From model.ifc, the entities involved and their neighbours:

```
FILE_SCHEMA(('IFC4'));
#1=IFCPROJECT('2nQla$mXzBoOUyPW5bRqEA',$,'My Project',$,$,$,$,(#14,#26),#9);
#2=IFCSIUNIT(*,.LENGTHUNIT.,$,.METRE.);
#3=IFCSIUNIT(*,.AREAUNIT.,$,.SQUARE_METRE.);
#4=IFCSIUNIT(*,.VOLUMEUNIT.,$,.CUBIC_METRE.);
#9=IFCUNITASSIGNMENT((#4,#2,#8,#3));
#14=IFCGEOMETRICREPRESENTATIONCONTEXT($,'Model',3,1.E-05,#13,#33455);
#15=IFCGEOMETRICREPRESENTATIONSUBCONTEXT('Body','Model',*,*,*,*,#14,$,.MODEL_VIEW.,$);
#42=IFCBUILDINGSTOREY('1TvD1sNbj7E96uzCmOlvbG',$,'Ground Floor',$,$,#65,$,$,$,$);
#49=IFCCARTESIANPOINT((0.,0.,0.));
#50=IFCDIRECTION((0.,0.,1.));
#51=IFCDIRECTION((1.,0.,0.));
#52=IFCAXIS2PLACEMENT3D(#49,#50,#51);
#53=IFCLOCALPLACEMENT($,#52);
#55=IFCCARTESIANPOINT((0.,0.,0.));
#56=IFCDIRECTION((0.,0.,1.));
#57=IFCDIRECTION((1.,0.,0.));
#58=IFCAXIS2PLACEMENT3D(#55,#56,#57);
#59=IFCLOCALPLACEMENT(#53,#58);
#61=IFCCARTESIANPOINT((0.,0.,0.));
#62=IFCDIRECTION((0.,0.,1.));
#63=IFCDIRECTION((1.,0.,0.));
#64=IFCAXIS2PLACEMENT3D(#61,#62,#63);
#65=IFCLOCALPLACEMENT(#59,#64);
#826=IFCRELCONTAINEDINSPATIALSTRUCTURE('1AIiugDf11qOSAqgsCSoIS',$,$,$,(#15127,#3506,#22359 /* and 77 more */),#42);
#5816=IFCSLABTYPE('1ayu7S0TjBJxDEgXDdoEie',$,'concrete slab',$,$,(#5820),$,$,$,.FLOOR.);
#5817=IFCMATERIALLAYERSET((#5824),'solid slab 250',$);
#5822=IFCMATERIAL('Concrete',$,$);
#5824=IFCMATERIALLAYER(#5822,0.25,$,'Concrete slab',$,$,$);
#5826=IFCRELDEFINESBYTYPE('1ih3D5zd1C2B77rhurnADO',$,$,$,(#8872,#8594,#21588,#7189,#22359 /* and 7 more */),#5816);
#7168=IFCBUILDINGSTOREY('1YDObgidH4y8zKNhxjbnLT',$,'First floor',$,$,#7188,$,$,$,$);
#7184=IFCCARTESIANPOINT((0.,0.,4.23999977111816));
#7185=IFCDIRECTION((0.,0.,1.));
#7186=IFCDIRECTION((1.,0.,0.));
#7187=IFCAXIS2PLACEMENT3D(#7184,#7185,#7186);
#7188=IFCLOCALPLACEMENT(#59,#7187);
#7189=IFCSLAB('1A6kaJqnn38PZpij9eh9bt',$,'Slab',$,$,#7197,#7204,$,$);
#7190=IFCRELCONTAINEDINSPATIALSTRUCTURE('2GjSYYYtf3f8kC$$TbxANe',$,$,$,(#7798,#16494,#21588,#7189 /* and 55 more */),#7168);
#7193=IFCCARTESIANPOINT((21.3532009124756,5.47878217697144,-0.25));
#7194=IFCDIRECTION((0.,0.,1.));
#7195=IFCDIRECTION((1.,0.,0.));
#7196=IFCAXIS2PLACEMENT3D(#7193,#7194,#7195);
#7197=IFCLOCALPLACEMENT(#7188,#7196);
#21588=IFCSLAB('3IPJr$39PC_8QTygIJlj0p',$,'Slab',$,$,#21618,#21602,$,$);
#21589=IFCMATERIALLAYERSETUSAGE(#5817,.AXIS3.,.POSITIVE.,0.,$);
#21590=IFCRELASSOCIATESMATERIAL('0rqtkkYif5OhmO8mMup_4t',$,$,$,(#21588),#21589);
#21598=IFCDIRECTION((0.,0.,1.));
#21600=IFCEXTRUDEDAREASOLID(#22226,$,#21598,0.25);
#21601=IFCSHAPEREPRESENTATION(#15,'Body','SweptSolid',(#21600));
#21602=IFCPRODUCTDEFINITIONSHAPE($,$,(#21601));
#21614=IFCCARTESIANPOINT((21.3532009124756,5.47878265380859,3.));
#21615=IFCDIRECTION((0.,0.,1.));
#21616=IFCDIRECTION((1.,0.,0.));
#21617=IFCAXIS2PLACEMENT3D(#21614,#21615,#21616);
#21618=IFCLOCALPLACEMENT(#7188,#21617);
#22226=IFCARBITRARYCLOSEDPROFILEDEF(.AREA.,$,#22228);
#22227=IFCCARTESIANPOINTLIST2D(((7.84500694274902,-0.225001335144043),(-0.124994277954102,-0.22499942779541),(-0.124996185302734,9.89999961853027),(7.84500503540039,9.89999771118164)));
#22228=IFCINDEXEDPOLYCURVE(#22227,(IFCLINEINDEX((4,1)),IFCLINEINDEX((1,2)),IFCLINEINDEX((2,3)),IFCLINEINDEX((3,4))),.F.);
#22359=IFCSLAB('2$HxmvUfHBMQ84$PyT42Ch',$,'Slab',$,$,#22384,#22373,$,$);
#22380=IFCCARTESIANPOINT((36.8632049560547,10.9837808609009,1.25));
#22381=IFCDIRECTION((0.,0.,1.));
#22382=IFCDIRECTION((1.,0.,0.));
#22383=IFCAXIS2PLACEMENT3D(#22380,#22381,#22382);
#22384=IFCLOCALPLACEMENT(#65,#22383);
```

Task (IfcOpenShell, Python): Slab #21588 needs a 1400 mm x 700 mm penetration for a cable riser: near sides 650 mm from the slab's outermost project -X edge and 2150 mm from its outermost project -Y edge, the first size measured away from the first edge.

```python
import numpy as np
import ifcopenshell
import ifcopenshell.api.feature
import ifcopenshell.api.geometry
import ifcopenshell.api.root
import ifcopenshell.geom
import ifcopenshell.util.placement
import ifcopenshell.util.representation
import ifcopenshell.util.shape
import ifcopenshell.util.unit

model = ifcopenshell.open("model.ifc")
unit_scale = ifcopenshell.util.unit.calculate_unit_scale(model)
settings = ifcopenshell.geom.settings()


def volume(element):
    """Net volume in cubic metres, openings subtracted."""
    shape = ifcopenshell.geom.create_shape(settings, element)
    return ifcopenshell.util.shape.get_volume(shape.geometry)


slab = model.by_id(21588)
before = volume(slab)

# Extent in the slab's own axes, in metres. The edges named are its -X and -Y sides.
slab_shape = ifcopenshell.geom.create_shape(settings, slab)
vertices = ifcopenshell.util.shape.get_vertices(slab_shape.geometry)
x_min, y_min, bottom = vertices.min(axis=0)
top = vertices[:, 2].max()

opening = ifcopenshell.api.root.create_entity(model, ifc_class="IfcOpeningElement", name="Cable riser opening", predefined_type="OPENING")
context = ifcopenshell.util.representation.get_context(model, "Model", "Body", "MODEL_VIEW")
width, depth = 1.4, 0.7
outline = [(0.0, 0.0), (width, 0.0), (width, depth), (0.0, depth), (0.0, 0.0)]
# Overshoot both faces by 50 mm so the cut is clean.
shape = ifcopenshell.api.geometry.add_slab_representation(
    model, context=context, depth=top - bottom + 0.1, polyline=outline
)
ifcopenshell.api.geometry.assign_representation(model, product=opening, representation=shape)

matrix = ifcopenshell.util.placement.get_local_placement(slab.ObjectPlacement)
matrix[:, 3] = matrix @ np.append(np.array([x_min + 0.65, y_min + 2.15, bottom - 0.05]) / unit_scale, 1.0)
ifcopenshell.api.geometry.edit_object_placement(model, product=opening, matrix=matrix, is_si=False)
ifcopenshell.api.feature.add_feature(model, feature=opening, element=slab)

after = volume(slab)

print(f"slab volume {before:.3f} -> {after:.3f} m3")

model.write("model_updated.ifc")
```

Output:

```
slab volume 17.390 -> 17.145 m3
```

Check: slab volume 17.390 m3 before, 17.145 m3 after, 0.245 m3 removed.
